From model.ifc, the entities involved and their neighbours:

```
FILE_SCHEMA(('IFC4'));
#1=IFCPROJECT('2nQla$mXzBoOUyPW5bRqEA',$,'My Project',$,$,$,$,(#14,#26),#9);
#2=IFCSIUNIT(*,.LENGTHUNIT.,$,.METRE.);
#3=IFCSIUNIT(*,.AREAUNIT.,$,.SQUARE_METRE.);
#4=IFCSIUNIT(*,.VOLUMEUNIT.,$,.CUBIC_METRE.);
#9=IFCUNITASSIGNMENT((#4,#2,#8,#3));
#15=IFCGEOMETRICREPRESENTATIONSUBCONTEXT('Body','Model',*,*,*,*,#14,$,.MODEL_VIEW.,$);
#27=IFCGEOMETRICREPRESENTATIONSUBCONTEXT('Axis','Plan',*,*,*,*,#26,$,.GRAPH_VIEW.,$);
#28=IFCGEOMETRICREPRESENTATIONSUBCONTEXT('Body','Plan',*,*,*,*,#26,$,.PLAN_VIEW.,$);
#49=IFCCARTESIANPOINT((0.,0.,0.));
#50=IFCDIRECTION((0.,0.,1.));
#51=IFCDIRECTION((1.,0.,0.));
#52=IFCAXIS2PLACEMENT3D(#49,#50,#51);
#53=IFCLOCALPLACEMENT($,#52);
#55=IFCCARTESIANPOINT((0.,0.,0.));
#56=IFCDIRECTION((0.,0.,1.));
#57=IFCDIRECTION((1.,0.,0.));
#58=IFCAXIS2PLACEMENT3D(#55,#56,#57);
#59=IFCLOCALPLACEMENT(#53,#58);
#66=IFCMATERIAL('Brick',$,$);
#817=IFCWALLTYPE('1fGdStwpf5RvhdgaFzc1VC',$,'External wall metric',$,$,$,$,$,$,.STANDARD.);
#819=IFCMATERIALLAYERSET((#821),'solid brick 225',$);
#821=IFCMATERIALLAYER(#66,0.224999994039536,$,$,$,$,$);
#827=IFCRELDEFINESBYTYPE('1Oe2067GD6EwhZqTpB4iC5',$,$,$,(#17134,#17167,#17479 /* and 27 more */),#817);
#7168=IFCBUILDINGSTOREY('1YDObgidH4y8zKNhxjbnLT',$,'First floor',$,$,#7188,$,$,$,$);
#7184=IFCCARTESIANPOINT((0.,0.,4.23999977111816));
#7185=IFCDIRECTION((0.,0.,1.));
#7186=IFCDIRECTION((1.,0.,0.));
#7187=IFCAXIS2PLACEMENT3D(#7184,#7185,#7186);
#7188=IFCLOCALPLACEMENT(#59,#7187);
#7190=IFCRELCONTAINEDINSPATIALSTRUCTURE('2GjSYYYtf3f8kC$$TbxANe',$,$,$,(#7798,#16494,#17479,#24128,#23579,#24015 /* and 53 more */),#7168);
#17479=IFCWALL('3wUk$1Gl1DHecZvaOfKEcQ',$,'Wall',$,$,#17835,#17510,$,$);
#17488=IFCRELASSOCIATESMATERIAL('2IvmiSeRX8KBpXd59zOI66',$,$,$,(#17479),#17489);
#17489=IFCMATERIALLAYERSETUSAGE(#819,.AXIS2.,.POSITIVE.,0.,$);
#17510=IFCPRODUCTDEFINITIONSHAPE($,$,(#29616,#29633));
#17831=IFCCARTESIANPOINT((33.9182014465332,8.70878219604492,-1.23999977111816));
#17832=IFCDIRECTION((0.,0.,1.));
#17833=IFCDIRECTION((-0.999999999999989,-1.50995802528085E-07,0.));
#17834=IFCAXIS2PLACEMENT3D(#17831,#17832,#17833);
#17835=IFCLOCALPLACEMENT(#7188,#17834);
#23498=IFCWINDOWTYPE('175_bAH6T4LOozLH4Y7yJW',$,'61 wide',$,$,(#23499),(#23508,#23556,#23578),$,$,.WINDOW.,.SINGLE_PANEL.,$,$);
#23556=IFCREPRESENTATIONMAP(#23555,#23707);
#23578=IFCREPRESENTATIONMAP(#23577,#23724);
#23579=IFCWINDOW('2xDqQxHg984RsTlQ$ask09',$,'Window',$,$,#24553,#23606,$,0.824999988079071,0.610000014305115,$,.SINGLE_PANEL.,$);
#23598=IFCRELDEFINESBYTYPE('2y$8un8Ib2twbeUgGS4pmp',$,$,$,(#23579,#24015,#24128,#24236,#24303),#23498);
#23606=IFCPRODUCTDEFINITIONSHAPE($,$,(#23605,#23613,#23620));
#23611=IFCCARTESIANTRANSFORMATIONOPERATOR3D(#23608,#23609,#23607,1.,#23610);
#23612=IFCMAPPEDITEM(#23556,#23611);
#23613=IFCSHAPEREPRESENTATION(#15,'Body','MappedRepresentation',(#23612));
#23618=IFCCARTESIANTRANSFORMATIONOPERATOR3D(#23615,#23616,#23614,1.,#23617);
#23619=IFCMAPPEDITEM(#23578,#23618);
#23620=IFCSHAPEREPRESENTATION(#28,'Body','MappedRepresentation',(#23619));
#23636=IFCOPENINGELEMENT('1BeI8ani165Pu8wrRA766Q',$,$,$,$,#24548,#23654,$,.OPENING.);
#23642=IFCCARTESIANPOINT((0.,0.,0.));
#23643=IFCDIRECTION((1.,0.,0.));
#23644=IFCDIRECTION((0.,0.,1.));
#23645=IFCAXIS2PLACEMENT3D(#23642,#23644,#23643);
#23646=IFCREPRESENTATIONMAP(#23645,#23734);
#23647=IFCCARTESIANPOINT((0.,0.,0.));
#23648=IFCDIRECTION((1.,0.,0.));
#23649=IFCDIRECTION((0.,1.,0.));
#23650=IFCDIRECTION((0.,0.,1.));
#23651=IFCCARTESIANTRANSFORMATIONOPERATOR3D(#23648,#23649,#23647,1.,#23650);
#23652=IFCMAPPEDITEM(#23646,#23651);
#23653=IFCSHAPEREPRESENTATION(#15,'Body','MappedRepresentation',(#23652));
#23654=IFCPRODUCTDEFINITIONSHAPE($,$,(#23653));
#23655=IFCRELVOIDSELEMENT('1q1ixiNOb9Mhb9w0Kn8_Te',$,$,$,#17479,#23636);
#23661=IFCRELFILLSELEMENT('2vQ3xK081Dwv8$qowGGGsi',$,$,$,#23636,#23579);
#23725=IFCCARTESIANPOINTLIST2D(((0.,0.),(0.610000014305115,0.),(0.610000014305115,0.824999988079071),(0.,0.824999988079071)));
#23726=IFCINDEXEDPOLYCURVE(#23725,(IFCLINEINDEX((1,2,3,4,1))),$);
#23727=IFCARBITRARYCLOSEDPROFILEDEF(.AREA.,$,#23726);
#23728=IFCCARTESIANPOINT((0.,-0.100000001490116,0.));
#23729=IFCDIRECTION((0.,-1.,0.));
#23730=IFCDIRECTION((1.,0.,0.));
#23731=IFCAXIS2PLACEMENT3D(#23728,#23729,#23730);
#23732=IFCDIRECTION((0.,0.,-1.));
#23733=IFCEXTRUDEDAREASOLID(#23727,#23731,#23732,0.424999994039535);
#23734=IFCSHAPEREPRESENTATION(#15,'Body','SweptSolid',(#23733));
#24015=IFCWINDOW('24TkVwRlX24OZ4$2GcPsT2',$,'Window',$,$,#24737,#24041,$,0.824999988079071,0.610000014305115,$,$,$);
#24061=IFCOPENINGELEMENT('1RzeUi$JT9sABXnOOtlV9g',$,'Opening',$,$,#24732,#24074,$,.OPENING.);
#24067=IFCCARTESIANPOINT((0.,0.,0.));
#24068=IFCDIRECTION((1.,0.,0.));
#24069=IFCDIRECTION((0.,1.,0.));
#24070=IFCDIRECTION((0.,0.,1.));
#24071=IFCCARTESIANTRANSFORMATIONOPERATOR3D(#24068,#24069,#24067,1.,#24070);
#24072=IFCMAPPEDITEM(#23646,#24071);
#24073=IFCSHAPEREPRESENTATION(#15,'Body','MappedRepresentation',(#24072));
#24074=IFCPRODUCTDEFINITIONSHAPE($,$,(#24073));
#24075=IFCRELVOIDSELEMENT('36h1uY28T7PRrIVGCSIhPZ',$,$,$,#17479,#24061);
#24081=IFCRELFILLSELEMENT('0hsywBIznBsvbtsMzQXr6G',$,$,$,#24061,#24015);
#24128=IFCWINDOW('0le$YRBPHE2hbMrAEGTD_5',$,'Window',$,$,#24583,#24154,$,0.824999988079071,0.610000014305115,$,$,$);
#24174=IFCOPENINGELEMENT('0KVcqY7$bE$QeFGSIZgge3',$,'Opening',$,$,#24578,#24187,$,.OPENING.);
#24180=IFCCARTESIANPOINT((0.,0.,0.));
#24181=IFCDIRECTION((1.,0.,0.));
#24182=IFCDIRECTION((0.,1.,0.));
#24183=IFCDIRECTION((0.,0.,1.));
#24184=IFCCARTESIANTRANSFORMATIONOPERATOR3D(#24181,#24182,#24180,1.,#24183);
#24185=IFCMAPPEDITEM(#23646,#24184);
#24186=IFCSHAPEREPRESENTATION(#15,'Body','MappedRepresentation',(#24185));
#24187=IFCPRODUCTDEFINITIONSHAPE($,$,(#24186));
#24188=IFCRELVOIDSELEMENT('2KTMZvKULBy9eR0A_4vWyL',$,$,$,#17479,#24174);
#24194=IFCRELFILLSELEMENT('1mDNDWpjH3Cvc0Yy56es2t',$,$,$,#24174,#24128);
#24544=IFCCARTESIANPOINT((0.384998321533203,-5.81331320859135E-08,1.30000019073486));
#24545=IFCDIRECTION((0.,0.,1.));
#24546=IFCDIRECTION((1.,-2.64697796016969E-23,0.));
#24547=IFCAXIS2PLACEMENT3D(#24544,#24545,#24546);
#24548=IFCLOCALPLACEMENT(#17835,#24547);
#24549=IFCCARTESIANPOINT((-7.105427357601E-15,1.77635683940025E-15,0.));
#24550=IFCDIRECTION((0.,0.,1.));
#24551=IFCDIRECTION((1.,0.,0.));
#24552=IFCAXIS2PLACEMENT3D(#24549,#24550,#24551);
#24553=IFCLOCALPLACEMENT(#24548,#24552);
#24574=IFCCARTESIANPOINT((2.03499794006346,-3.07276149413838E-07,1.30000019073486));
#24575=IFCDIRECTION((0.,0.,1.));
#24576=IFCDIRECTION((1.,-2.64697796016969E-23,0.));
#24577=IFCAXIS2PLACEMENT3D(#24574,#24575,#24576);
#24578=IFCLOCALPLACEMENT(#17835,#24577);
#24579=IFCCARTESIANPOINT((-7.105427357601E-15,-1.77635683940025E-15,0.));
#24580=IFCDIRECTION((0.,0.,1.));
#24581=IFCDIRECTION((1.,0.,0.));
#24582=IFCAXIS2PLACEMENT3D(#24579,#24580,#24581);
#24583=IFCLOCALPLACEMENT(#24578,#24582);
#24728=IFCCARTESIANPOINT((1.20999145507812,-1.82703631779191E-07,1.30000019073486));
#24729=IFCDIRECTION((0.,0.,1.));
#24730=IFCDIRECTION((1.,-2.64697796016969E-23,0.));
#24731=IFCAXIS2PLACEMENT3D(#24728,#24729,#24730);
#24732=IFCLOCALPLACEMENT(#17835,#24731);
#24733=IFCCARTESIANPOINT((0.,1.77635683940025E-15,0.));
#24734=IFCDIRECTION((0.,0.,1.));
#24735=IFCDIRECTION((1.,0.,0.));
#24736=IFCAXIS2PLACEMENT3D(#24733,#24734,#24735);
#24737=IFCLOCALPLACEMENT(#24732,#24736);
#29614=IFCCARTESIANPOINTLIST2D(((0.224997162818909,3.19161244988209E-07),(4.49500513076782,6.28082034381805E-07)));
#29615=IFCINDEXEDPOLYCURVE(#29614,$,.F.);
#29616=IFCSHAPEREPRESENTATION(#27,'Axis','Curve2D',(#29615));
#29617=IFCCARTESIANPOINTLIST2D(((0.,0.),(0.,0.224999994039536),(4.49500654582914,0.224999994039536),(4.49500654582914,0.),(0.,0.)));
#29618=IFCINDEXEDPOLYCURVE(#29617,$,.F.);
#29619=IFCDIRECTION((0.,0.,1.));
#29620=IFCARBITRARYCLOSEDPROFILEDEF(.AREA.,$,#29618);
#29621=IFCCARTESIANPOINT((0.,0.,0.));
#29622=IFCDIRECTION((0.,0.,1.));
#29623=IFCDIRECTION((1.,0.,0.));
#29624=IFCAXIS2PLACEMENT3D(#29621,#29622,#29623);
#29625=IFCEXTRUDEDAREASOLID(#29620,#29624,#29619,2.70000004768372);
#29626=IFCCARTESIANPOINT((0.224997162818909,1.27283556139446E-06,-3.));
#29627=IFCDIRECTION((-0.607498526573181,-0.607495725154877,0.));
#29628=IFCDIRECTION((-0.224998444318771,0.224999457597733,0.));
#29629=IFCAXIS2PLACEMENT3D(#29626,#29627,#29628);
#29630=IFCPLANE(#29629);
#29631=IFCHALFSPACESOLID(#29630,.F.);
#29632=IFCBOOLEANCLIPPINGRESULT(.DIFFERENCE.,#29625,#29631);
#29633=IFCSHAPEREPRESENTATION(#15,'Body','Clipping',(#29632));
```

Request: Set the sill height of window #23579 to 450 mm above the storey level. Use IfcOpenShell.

```python
import numpy as np
import ifcopenshell
import ifcopenshell.api.geometry
import ifcopenshell.geom
import ifcopenshell.util.element
import ifcopenshell.util.placement
import ifcopenshell.util.shape
import ifcopenshell.util.unit

model = ifcopenshell.open("model.ifc")
unit_scale = ifcopenshell.util.unit.calculate_unit_scale(model)

window = model.by_guid("2xDqQxHg984RsTlQ$ask09")
opening = window.FillsVoids[0].RelatingOpeningElement
storey = ifcopenshell.util.element.get_container(window, ifc_class="IfcBuildingStorey")
level = ifcopenshell.util.placement.get_local_placement(storey.ObjectPlacement)[2, 3]

# The opening's origin need not be at the sill, so measure its lowest point.
shape = ifcopenshell.geom.create_shape(ifcopenshell.geom.settings(), opening)
bottom = ifcopenshell.util.shape.get_shape_bottom_elevation(shape, shape.geometry) / unit_scale
dz = level + 0.45 / unit_scale - bottom

shift = np.array([0.0, 0.0, dz])
# The window is placed relative to its opening, so it follows when the opening moves.
matrix = ifcopenshell.util.placement.get_local_placement(opening.ObjectPlacement)
matrix[:3, 3] += shift
ifcopenshell.api.geometry.edit_object_placement(
    model, product=opening, matrix=matrix, is_si=False, should_transform_children=True
)

print(f"moved by {dz * unit_scale:+.3f} m")

model.write("model_v2.ifc")
```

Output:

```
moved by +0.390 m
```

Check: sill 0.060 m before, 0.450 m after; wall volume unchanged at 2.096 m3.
